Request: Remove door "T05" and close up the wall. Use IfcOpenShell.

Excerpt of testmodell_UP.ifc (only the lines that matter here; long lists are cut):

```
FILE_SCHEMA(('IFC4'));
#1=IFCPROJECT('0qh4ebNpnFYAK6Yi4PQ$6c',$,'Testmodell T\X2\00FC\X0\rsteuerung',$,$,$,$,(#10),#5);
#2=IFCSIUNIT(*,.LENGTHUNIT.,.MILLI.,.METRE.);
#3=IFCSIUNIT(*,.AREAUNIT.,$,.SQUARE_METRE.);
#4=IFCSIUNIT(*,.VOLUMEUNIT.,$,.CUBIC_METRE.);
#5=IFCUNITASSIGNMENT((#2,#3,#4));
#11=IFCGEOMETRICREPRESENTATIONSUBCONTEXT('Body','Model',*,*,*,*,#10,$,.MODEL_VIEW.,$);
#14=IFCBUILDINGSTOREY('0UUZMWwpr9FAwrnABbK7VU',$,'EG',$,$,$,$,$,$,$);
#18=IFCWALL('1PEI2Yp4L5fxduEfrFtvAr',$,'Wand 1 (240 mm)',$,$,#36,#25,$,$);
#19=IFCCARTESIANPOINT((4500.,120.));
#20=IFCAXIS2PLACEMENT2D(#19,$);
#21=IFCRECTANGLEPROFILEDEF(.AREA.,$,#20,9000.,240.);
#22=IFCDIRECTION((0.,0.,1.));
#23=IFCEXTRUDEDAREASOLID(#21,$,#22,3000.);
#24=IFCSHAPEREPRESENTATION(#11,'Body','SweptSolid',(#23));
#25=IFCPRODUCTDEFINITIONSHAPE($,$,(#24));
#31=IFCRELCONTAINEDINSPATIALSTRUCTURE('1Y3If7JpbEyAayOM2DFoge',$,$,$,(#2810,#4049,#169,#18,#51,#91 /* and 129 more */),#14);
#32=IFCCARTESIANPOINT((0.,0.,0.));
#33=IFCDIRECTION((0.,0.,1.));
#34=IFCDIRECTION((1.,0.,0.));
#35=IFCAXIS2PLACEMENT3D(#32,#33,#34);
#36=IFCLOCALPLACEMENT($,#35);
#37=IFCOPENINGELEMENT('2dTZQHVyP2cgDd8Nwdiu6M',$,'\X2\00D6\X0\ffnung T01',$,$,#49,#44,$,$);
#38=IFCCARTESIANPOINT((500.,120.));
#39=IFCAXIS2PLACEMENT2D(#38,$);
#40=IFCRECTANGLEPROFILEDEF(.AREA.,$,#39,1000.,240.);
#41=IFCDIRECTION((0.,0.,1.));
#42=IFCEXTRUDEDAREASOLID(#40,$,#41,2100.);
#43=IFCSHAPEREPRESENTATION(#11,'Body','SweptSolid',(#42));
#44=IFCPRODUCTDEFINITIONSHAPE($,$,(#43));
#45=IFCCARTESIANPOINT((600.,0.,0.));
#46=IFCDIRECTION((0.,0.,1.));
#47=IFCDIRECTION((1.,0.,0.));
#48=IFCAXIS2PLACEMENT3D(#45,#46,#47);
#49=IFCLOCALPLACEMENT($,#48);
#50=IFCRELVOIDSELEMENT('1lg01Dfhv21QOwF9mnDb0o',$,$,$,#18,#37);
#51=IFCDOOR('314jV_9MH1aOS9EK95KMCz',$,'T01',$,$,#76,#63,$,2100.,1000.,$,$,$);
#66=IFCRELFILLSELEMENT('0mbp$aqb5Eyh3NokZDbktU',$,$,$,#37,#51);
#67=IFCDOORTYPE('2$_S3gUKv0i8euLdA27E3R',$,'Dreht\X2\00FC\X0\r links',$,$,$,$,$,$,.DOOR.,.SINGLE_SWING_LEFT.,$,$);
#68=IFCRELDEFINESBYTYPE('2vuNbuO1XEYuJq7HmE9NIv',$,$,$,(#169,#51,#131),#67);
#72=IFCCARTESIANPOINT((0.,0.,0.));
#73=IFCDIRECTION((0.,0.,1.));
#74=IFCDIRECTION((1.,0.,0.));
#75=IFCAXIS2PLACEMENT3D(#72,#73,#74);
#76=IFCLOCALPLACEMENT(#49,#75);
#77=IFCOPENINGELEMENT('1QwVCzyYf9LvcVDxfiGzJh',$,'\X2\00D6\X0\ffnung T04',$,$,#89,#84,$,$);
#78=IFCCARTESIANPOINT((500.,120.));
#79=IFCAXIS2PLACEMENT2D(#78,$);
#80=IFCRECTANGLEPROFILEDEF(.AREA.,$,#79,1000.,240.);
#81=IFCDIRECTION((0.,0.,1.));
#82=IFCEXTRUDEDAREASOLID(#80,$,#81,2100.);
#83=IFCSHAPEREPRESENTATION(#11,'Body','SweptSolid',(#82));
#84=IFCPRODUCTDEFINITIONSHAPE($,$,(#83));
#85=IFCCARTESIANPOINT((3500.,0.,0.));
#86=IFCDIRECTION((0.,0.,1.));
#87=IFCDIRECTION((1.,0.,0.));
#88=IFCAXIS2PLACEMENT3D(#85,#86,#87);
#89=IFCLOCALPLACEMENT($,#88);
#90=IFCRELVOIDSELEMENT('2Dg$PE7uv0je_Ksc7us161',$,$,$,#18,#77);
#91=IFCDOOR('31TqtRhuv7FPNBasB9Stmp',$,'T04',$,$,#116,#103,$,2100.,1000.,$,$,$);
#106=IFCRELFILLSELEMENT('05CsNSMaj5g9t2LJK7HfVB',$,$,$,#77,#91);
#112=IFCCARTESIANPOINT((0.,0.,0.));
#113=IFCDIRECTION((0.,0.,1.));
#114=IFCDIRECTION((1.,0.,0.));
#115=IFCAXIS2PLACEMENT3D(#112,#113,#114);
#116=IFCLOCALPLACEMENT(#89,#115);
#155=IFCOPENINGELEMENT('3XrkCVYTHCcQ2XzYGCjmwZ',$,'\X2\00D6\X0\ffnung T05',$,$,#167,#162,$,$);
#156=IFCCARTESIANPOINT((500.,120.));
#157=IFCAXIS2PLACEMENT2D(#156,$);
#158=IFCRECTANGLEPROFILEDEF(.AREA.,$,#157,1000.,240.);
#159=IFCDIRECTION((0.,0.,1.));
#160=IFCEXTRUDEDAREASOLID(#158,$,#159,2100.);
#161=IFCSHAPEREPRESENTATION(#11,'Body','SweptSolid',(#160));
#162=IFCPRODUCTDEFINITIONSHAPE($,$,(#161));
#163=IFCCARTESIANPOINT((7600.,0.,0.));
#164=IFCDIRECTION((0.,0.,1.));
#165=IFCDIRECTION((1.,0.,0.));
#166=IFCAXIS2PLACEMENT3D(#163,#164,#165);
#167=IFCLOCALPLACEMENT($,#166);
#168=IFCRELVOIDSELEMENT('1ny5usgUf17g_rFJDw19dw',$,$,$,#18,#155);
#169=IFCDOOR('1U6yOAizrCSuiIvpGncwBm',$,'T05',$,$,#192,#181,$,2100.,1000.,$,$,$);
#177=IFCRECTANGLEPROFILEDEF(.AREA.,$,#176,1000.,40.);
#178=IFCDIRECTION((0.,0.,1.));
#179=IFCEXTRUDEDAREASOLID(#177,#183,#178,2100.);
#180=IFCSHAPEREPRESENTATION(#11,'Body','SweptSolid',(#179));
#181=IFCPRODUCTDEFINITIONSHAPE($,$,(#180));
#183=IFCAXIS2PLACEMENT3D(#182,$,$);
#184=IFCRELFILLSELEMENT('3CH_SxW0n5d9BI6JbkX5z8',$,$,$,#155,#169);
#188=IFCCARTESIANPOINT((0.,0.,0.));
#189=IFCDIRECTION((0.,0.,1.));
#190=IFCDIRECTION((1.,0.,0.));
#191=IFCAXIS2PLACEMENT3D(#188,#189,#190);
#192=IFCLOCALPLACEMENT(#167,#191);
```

```python
import ifcopenshell
import ifcopenshell.api.feature
import ifcopenshell.api.root
import ifcopenshell.geom
import ifcopenshell.util.shape

model = ifcopenshell.open("testmodell_UP.ifc")
settings = ifcopenshell.geom.settings()


def volume(element):
    """Net volume in cubic metres, openings subtracted."""
    shape = ifcopenshell.geom.create_shape(settings, element)
    return ifcopenshell.util.shape.get_volume(shape.geometry)


door = model.by_guid("1U6yOAizrCSuiIvpGncwBm")
opening = door.FillsVoids[0].RelatingOpeningElement
wall = opening.VoidsElements[0].RelatingBuildingElement
before = volume(wall)

ifcopenshell.api.root.remove_product(model, product=door)
ifcopenshell.api.feature.remove_feature(model, feature=opening)

after = volume(wall)

print(f"wall volume {before:.3f} -> {after:.3f} m3")

model.write("testmodell_UP_rev.ifc")
```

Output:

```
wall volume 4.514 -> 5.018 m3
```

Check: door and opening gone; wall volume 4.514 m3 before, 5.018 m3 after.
